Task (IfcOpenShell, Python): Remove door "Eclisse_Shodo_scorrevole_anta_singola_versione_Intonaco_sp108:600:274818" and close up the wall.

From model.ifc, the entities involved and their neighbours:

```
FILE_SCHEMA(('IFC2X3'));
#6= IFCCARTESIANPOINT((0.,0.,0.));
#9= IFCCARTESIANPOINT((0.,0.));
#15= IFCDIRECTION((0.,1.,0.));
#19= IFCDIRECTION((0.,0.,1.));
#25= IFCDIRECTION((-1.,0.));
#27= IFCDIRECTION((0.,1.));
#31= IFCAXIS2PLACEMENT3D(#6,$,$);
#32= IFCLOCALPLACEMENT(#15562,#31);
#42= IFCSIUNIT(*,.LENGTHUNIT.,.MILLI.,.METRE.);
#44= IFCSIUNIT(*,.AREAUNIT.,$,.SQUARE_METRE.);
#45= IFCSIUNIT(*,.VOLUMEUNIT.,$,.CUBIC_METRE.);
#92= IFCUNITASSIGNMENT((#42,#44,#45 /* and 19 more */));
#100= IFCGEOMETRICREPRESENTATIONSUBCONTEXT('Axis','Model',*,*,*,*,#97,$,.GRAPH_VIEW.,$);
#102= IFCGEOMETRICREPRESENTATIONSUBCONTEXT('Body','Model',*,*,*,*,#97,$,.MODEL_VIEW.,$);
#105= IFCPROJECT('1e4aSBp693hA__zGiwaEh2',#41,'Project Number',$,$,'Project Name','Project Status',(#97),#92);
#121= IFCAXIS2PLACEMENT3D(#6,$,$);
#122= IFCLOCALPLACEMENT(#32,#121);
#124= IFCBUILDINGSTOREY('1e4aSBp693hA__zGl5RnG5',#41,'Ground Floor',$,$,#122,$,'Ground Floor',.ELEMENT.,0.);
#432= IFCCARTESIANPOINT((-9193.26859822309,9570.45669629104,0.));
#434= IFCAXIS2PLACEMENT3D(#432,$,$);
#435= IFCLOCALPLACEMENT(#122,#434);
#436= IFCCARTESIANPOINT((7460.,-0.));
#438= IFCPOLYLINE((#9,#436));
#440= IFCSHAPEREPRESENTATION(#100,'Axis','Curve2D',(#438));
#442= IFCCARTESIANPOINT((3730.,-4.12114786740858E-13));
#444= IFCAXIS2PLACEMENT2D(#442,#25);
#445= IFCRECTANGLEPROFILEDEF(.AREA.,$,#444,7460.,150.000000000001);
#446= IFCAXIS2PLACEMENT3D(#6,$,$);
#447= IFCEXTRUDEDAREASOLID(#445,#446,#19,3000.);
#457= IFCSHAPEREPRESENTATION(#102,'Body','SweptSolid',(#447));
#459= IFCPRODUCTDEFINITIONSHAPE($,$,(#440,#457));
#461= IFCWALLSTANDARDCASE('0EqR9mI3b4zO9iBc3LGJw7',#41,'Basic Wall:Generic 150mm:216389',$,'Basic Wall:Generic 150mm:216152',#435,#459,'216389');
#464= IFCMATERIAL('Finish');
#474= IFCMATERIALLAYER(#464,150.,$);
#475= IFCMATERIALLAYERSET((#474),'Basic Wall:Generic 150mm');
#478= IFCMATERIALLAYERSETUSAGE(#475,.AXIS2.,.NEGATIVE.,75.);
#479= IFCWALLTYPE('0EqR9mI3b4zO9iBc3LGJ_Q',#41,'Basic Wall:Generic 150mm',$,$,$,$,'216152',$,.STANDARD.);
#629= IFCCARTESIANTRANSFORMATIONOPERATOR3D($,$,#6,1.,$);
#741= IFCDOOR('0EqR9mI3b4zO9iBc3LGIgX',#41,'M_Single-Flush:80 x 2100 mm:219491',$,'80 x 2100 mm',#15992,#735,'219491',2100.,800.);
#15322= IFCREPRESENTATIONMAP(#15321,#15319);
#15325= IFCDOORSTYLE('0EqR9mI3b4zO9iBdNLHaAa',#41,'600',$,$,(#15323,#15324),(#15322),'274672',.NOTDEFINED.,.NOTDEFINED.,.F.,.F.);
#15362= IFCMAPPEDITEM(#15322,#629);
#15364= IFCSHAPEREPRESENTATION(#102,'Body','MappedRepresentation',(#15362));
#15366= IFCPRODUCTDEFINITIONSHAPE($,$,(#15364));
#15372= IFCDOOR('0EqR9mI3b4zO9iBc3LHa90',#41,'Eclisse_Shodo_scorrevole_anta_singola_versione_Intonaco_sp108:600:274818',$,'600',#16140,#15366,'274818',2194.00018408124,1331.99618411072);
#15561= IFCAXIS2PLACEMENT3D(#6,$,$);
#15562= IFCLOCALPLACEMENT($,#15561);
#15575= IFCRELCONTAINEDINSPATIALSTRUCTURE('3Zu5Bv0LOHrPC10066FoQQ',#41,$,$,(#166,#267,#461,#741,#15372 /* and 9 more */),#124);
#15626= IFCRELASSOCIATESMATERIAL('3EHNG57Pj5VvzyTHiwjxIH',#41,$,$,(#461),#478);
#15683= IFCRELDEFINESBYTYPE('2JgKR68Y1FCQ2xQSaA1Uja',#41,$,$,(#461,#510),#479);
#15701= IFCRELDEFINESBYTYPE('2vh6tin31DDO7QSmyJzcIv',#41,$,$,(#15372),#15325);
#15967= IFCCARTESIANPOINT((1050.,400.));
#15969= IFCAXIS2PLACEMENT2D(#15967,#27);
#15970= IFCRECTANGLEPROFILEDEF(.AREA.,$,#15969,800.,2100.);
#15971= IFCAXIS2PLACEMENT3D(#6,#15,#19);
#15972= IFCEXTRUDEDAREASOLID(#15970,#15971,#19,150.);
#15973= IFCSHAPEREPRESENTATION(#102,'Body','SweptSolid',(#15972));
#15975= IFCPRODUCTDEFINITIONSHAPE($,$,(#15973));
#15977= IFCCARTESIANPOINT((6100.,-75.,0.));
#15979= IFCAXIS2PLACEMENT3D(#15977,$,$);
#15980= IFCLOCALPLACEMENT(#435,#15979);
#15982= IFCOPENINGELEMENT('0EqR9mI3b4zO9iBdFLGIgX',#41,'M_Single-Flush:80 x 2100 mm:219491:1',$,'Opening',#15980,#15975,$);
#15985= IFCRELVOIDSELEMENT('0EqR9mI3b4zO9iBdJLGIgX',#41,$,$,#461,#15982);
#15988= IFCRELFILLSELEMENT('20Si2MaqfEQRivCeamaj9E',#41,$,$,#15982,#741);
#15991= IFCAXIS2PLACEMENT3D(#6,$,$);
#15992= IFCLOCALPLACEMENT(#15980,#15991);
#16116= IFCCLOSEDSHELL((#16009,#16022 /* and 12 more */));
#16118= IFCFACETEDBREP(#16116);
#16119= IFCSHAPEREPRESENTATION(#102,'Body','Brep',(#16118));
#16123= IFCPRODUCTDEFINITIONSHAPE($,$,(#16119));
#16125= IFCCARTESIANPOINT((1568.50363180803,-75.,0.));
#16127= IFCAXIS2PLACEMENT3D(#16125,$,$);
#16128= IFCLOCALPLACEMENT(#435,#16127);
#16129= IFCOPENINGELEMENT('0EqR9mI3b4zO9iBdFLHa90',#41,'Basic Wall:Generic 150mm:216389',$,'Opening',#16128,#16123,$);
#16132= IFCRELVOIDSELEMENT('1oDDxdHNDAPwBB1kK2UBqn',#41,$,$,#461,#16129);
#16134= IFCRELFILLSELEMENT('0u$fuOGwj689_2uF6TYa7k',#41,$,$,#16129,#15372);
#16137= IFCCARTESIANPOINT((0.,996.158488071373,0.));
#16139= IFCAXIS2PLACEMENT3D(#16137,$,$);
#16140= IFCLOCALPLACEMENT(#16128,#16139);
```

```python
import ifcopenshell
import ifcopenshell.api.feature
import ifcopenshell.api.root
import ifcopenshell.geom
import ifcopenshell.util.shape

model = ifcopenshell.open("model.ifc")
settings = ifcopenshell.geom.settings()


def volume(element):
    """Net volume in cubic metres, openings subtracted."""
    shape = ifcopenshell.geom.create_shape(settings, element)
    return ifcopenshell.util.shape.get_volume(shape.geometry)


door = model.by_guid("0EqR9mI3b4zO9iBc3LHa90")
opening = door.FillsVoids[0].RelatingOpeningElement
wall = opening.VoidsElements[0].RelatingBuildingElement
before = volume(wall)

ifcopenshell.api.root.remove_product(model, product=door)
ifcopenshell.api.feature.remove_feature(model, feature=opening)

after = volume(wall)

print(f"wall volume {before:.3f} -> {after:.3f} m3")

model.write("model_v2.ifc")
```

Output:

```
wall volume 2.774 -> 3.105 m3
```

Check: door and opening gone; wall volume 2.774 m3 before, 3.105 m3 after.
